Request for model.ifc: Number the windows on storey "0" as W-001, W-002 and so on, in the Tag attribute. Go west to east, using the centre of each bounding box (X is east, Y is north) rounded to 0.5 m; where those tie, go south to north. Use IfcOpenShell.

First a look at what the model holds.

```python
import ifcopenshell
import ifcopenshell.util.element
import ifcopenshell.util.placement

model = ifcopenshell.open("model.ifc")
print(model.schema)
storey = next(s for s in model.by_type("IfcBuildingStorey") if s.Name == "0")
windows = [e for e in ifcopenshell.util.element.get_decomposition(storey) if e.is_a("IfcWindow")]
for e in sorted(windows, key=lambda e: e.id()):
    origin = ifcopenshell.util.placement.get_local_placement(e.ObjectPlacement)[:3, 3]
    print(e.id(), e.Tag, e.Name, origin.round(2) + 0.0, sep=" | ")
```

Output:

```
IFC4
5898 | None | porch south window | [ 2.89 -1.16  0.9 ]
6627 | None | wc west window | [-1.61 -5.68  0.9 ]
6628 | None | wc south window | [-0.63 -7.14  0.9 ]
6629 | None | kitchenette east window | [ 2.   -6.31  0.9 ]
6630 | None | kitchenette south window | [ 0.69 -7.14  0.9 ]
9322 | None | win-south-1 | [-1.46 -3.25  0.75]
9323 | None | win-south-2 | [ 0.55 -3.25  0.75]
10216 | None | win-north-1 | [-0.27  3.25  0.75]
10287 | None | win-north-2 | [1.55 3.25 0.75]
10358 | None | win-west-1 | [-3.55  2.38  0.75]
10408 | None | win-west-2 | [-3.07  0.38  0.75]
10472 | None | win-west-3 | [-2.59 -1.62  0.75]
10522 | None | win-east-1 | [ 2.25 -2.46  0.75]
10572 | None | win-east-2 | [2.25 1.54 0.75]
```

```python
import ifcopenshell
import ifcopenshell.geom
import ifcopenshell.util.element
import ifcopenshell.util.shape

model = ifcopenshell.open("model.ifc")
settings = ifcopenshell.geom.settings()
settings.set("use-world-coords", True)


def centre(element):
    shape = ifcopenshell.geom.create_shape(settings, element)
    return ifcopenshell.util.shape.get_bbox_centroid(shape.geometry)


storey = next(s for s in model.by_type("IfcBuildingStorey") if s.Name == "0")
windows = [e for e in ifcopenshell.util.element.get_decomposition(storey) if e.is_a("IfcWindow")]

# Insertion points can sit at a corner or the storey origin, so sort by the geometry (in metres).
centres = {e: centre(e) for e in windows}
windows.sort(key=lambda e: (round(centres[e][0] / 0.5), centres[e][1]))

for i, e in enumerate(windows, start=1):
    number = f"W-0{i:02d}"
    e.Tag = number
    print(e.id(), number)

model.write("model_edited.ifc")
```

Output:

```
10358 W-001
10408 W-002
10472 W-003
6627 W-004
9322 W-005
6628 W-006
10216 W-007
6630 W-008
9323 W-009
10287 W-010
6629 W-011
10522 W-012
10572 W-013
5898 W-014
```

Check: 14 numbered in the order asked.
